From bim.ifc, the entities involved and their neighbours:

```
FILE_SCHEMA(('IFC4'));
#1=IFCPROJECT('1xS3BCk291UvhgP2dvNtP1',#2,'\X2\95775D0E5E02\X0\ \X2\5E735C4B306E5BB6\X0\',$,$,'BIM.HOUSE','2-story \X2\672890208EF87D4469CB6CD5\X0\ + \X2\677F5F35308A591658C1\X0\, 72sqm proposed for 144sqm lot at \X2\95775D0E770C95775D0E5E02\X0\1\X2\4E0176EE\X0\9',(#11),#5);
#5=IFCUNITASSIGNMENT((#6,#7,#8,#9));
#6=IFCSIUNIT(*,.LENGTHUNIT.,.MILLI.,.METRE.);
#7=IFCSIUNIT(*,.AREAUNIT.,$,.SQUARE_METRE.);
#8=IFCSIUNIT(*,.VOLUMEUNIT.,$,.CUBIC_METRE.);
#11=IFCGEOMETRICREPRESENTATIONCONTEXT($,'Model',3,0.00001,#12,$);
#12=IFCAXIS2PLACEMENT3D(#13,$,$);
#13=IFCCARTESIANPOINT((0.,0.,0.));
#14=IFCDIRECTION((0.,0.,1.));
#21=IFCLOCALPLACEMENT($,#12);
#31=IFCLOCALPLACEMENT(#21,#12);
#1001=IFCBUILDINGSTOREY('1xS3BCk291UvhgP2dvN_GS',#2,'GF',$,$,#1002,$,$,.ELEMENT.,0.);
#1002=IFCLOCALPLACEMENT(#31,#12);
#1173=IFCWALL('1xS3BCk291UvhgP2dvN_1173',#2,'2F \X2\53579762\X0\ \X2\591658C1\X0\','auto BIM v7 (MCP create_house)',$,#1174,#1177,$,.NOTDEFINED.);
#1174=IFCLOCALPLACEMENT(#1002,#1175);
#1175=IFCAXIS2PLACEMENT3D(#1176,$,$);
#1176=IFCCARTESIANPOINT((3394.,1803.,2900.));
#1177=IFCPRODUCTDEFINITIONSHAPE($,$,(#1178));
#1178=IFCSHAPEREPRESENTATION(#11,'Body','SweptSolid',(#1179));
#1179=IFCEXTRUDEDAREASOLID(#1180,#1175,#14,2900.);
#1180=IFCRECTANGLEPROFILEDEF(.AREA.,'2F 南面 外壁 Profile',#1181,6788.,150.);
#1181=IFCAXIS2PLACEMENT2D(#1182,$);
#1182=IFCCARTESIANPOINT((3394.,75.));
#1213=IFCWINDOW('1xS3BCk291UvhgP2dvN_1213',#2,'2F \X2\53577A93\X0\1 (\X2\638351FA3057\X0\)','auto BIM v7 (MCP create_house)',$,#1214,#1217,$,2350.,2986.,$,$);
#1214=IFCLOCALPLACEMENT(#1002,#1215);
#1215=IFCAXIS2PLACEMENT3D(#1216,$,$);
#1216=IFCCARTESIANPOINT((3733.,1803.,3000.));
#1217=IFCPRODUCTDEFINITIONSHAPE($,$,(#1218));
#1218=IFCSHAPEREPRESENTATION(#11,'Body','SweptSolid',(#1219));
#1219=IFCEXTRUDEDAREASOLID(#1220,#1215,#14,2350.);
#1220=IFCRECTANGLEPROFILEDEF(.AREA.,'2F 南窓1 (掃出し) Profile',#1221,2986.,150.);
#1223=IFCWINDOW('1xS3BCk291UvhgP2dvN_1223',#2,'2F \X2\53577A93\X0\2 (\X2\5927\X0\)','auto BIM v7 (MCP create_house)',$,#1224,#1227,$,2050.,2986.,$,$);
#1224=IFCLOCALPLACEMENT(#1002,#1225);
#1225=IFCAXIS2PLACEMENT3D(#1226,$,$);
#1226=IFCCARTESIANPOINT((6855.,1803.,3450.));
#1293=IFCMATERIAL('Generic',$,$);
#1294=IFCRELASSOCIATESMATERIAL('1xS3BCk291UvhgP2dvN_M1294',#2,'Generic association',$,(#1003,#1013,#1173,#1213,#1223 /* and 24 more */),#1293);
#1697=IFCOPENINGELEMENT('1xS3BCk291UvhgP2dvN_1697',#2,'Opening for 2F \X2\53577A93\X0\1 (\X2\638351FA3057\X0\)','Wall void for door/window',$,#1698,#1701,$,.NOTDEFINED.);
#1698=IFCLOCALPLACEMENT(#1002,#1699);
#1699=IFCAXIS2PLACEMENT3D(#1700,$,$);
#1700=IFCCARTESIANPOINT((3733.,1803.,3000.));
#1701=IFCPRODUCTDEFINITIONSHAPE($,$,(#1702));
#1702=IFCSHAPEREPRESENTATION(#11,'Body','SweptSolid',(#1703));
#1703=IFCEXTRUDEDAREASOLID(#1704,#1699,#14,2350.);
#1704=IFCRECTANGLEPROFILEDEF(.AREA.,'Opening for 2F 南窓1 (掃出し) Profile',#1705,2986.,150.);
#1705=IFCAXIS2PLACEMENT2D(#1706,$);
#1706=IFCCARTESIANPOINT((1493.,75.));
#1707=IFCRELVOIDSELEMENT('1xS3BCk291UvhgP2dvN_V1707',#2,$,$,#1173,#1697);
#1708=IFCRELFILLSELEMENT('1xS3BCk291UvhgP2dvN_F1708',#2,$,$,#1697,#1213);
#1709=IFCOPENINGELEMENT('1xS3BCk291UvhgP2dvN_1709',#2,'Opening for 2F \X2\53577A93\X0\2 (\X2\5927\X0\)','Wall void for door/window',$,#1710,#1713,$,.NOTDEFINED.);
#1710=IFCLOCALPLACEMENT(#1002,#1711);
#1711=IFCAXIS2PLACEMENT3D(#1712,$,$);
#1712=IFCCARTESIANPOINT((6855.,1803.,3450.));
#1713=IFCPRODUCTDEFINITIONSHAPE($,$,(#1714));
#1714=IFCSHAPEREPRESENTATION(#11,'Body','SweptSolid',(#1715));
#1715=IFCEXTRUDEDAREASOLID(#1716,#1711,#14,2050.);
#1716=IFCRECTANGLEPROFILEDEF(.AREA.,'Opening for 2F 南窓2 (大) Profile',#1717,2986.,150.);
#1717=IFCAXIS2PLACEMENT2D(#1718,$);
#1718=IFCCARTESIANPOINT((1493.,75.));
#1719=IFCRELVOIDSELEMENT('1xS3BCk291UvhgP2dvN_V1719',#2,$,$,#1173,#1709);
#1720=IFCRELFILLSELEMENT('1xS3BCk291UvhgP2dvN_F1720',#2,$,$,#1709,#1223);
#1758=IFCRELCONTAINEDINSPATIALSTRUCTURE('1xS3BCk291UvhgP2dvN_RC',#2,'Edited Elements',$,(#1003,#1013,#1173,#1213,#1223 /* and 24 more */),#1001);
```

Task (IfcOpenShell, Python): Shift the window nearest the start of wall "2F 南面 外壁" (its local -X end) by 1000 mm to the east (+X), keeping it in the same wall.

```python
import ifcopenshell
import ifcopenshell.api.geometry
import ifcopenshell.util.placement
import ifcopenshell.util.unit

model = ifcopenshell.open("bim.ifc")
unit_scale = ifcopenshell.util.unit.calculate_unit_scale(model)

window = model.by_id(1213)
opening = window.FillsVoids[0].RelatingOpeningElement
wall = opening.VoidsElements[0].RelatingBuildingElement

wall_matrix = ifcopenshell.util.placement.get_local_placement(wall.ObjectPlacement)
shift = wall_matrix[:3, 0] * 1 / unit_scale
before = ifcopenshell.util.placement.get_local_placement(window.ObjectPlacement)[:3, 3].copy()

# The window is not placed relative to its opening, so move both.
for product in (opening, window):
    matrix = ifcopenshell.util.placement.get_local_placement(product.ObjectPlacement)
    matrix[:3, 3] += shift
    ifcopenshell.api.geometry.edit_object_placement(model, product=product, matrix=matrix, is_si=False)

after = ifcopenshell.util.placement.get_local_placement(window.ObjectPlacement)[:3, 3]
print("window moved by", (after - before).round(3) + 0.0)

model.write("bim_edited.ifc")
```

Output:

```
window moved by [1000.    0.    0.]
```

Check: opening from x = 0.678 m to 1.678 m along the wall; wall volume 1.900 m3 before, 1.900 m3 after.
